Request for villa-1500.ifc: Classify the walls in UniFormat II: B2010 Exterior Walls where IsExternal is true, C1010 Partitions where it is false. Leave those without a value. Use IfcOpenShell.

First a look at what the model holds.

```python
import ifcopenshell
import ifcopenshell.util.element

model = ifcopenshell.open("villa-1500.ifc")
print(model.schema)
print("classifications:", [c.Name for c in model.by_type("IfcClassification")])
values = [ifcopenshell.util.element.get_pset(e, "Pset_WallCommon", "IsExternal") for e in model.by_type("IfcWall")]
for value in (True, False, None):
    print("IsExternal", value, values.count(value))
```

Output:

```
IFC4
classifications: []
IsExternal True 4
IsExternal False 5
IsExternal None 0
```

```python
import ifcopenshell
import ifcopenshell.api.classification
import ifcopenshell.util.element

model = ifcopenshell.open("villa-1500.ifc")

system = ifcopenshell.api.classification.add_classification(model, classification="UniFormat II")

walls = model.by_type("IfcWall")
external = {e: ifcopenshell.util.element.get_pset(e, "Pset_WallCommon", "IsExternal") for e in walls}
for flag, code, name in ((True, "B2010", "Exterior Walls"), (False, "C1010", "Partitions")):
    products = [e for e in walls if external[e] is flag]
    ifcopenshell.api.classification.add_reference(
        model, products=products, classification=system, identification=code, name=name
    )
    print(code, len(products))

model.write("villa-1500_rev.ifc")
```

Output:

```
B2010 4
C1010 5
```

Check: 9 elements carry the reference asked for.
